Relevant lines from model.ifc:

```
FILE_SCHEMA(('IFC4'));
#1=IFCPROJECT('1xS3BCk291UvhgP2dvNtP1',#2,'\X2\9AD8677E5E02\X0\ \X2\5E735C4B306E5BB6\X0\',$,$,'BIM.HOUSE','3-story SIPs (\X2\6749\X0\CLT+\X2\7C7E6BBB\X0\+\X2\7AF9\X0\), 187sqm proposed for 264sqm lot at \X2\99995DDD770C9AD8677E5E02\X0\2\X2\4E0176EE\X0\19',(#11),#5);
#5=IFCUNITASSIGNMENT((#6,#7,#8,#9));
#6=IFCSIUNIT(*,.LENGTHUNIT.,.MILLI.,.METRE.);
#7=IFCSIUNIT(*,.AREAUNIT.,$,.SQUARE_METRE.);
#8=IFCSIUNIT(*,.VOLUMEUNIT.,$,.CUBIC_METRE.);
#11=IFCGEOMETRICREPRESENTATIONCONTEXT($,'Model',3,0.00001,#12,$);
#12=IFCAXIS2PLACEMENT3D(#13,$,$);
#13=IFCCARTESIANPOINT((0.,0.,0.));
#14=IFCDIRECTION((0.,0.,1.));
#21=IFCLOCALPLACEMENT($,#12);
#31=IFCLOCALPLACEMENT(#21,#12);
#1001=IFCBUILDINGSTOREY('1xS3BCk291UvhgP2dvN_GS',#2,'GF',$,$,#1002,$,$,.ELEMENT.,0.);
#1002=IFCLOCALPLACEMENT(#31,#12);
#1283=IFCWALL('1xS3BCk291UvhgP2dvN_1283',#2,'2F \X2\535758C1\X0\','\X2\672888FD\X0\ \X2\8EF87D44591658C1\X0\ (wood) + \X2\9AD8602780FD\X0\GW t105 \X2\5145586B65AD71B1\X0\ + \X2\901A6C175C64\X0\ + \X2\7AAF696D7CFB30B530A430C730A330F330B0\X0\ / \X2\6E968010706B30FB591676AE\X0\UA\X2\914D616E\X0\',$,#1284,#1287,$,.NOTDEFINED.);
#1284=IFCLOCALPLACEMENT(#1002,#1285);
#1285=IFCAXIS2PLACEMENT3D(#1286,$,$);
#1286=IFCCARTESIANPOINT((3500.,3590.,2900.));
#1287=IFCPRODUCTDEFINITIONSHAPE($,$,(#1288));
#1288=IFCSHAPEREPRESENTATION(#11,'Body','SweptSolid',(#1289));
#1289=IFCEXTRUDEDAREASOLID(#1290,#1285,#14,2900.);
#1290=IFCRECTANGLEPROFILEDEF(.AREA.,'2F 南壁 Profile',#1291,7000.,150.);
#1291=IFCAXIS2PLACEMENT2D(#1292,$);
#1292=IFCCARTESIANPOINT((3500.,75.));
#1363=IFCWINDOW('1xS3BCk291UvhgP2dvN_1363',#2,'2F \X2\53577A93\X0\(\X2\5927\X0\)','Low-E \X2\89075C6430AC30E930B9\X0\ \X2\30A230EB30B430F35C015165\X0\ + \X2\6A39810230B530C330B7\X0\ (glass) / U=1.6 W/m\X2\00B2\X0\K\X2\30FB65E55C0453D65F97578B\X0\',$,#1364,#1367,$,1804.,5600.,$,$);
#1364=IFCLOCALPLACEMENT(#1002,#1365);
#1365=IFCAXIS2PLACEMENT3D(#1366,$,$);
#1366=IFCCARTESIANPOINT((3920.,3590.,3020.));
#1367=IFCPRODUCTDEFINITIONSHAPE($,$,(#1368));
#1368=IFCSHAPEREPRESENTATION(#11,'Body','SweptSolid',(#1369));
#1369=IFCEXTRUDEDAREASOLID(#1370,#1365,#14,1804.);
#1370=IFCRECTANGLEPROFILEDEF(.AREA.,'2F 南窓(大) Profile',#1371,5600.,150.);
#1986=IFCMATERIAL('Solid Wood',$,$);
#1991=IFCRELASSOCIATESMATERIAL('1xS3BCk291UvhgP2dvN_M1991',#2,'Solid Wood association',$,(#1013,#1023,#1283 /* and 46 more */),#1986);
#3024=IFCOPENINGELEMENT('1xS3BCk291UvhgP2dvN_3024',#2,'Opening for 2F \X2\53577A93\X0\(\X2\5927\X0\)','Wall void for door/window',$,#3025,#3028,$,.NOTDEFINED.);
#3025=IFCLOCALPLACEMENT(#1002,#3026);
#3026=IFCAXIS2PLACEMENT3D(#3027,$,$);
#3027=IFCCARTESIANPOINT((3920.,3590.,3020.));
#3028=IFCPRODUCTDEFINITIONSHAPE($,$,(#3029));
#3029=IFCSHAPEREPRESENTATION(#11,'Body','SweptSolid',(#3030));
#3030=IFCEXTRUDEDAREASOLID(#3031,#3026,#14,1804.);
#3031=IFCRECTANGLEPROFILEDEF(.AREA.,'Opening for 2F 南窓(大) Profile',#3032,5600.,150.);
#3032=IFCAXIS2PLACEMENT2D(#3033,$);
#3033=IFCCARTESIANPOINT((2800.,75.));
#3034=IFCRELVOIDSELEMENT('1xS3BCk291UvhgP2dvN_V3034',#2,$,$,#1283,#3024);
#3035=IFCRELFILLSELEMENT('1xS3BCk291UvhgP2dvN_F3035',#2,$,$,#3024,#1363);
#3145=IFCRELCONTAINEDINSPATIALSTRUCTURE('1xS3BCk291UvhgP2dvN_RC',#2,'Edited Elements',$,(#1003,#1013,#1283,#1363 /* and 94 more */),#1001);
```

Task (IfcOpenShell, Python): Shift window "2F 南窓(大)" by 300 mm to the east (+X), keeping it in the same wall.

```python
import ifcopenshell
import ifcopenshell.api.geometry
import ifcopenshell.util.placement
import ifcopenshell.util.unit

model = ifcopenshell.open("model.ifc")
unit_scale = ifcopenshell.util.unit.calculate_unit_scale(model)

window = model.by_guid("1xS3BCk291UvhgP2dvN_1363")
opening = window.FillsVoids[0].RelatingOpeningElement
wall = opening.VoidsElements[0].RelatingBuildingElement

wall_matrix = ifcopenshell.util.placement.get_local_placement(wall.ObjectPlacement)
shift = wall_matrix[:3, 0] * 0.3 / unit_scale
before = ifcopenshell.util.placement.get_local_placement(window.ObjectPlacement)[:3, 3].copy()

# The window is not placed relative to its opening, so move both.
for product in (opening, window):
    matrix = ifcopenshell.util.placement.get_local_placement(product.ObjectPlacement)
    matrix[:3, 3] += shift
    ifcopenshell.api.geometry.edit_object_placement(model, product=product, matrix=matrix, is_si=False)

after = ifcopenshell.util.placement.get_local_placement(window.ObjectPlacement)[:3, 3]
print("window moved by", (after - before).round(3) + 0.0)

model.write("model_rev.ifc")
```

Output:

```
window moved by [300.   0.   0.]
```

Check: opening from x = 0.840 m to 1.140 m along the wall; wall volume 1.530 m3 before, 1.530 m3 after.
